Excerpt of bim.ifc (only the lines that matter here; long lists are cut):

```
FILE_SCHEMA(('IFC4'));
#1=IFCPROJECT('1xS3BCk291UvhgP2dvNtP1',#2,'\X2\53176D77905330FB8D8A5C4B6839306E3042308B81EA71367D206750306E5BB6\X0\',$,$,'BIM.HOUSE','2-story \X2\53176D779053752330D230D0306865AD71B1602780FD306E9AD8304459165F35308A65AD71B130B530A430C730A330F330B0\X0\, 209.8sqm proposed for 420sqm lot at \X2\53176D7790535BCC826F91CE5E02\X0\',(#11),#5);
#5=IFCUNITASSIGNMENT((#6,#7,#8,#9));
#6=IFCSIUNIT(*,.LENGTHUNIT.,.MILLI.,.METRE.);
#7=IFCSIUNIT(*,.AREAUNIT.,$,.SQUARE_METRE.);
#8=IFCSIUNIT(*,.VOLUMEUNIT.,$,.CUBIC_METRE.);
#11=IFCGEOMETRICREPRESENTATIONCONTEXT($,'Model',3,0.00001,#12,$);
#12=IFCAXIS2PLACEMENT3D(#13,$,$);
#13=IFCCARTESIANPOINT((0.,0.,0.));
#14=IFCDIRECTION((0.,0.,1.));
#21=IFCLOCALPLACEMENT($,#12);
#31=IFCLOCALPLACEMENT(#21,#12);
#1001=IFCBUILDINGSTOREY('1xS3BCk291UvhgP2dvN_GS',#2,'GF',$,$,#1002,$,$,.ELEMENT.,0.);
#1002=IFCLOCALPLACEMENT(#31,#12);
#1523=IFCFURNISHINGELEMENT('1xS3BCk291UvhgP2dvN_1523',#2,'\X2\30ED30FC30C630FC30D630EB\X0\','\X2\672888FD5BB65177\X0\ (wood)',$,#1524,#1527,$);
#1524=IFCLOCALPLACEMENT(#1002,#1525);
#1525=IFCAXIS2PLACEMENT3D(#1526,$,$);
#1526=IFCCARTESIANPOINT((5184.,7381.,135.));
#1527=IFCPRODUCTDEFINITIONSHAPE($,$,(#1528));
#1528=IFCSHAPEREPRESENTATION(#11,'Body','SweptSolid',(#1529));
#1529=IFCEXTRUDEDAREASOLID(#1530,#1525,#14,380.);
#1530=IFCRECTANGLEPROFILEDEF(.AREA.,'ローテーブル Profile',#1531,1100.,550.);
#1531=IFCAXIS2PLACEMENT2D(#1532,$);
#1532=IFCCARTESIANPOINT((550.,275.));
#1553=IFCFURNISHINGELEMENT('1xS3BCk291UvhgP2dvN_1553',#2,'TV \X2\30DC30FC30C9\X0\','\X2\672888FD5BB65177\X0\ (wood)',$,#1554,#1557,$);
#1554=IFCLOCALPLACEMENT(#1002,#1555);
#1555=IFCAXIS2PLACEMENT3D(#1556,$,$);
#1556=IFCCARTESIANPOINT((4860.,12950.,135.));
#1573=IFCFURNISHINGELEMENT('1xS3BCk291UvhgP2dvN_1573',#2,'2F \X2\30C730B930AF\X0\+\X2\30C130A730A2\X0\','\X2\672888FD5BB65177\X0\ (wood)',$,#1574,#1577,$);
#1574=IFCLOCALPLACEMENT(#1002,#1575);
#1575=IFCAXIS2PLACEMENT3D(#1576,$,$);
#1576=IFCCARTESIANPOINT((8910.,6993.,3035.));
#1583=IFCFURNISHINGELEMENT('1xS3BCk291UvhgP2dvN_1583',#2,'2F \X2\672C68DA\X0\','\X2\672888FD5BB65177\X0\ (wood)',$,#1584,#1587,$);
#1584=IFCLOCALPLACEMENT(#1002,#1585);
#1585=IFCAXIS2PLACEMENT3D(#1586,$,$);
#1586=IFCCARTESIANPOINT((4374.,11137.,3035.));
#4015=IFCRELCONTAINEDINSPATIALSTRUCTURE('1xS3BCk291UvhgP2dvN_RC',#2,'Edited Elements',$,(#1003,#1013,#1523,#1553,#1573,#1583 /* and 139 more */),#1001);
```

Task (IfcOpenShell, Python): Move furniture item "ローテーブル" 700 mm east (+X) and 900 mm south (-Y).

```python
import ifcopenshell
import ifcopenshell.api.geometry
import ifcopenshell.util.placement
import ifcopenshell.util.unit

model = ifcopenshell.open("bim.ifc")
unit_scale = ifcopenshell.util.unit.calculate_unit_scale(model)

item = model.by_guid("1xS3BCk291UvhgP2dvN_1523")
matrix = ifcopenshell.util.placement.get_local_placement(item.ObjectPlacement)
matrix[0, 3] += 0.7 / unit_scale
matrix[1, 3] -= 0.9 / unit_scale
ifcopenshell.api.geometry.edit_object_placement(model, product=item, matrix=matrix, is_si=False)

print(ifcopenshell.util.placement.get_local_placement(item.ObjectPlacement).round(3) + 0.0)

model.write("bim-out.ifc")
```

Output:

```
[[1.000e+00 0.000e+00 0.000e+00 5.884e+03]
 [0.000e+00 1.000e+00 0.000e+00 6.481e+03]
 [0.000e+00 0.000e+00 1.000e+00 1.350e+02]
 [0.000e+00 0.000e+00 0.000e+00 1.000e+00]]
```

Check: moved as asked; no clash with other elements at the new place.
